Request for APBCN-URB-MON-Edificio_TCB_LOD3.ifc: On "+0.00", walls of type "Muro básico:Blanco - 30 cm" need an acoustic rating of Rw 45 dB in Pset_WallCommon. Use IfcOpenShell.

First a look at what the model holds.

```python
import ifcopenshell
import ifcopenshell.util.element

model = ifcopenshell.open("APBCN-URB-MON-Edificio_TCB_LOD3.ifc")
print(model.schema)
storey = next(s for s in model.by_type("IfcBuildingStorey") if s.Name == "+0.00")
walls = [e for e in ifcopenshell.util.element.get_decomposition(storey) if e.is_a("IfcWall")]
seen = {}
for e in walls:
    element_type = ifcopenshell.util.element.get_type(e)
    key = (element_type.Name if element_type != e and element_type else None, ifcopenshell.util.element.get_pset(e, "Pset_WallCommon", "AcousticRating"))
    seen[key] = seen.get(key, 0) + 1
for (name, value), count in sorted(seen.items(), key=str):
    print(count, "x", name, "|", value)
```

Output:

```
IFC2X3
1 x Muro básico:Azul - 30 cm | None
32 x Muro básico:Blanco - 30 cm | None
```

```python
import ifcopenshell
import ifcopenshell.api.pset
import ifcopenshell.util.element

model = ifcopenshell.open("APBCN-URB-MON-Edificio_TCB_LOD3.ifc")

storey = next(s for s in model.by_type("IfcBuildingStorey") if s.Name == "+0.00")
walls = [e for e in ifcopenshell.util.element.get_decomposition(storey) if e.is_a("IfcWall")]

count = 0
for e in walls:
    element_type = ifcopenshell.util.element.get_type(e)
    if element_type in (None, e) or element_type.Name != "Muro básico:Blanco - 30 cm":
        continue
    # add_pset returns the element's existing set when there is one.
    pset = ifcopenshell.api.pset.add_pset(model, product=e, name="Pset_WallCommon")
    ifcopenshell.api.pset.edit_pset(model, pset=pset, properties={"AcousticRating": "Rw 45 dB"})
    count += 1

print(count, "walls updated")

model.write("APBCN-URB-MON-Edificio_TCB_LOD3_v2.ifc")
```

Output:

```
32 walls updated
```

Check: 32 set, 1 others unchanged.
